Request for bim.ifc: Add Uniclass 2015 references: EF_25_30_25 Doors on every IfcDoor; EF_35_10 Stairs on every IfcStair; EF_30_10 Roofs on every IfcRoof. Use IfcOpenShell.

First a look at what the model holds.

```python
import ifcopenshell

model = ifcopenshell.open("bim.ifc")
print(model.schema)
print("classifications:", [c.Name for c in model.by_type("IfcClassification")])
for ifc_class in ("IfcDoor", "IfcRoof", "IfcStair", "IfcWall", "IfcWindow"):
    print(ifc_class, len(model.by_type(ifc_class)))
```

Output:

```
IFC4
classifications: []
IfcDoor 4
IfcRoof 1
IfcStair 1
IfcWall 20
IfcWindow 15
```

```python
import ifcopenshell
import ifcopenshell.api.classification

model = ifcopenshell.open("bim.ifc")

system = ifcopenshell.api.classification.add_classification(model, classification="Uniclass 2015")

codes = {
    "IfcDoor": ("EF_25_30_25", "Doors"),
    "IfcStair": ("EF_35_10", "Stairs"),
    "IfcRoof": ("EF_30_10", "Roofs"),
}
for ifc_class, (code, name) in codes.items():
    products = model.by_type(ifc_class)
    ifcopenshell.api.classification.add_reference(
        model, products=products, classification=system, identification=code, name=name
    )
    print(code, len(products))

model.write("bim_rev.ifc")
```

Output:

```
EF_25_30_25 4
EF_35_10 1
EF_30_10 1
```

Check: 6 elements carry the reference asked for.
